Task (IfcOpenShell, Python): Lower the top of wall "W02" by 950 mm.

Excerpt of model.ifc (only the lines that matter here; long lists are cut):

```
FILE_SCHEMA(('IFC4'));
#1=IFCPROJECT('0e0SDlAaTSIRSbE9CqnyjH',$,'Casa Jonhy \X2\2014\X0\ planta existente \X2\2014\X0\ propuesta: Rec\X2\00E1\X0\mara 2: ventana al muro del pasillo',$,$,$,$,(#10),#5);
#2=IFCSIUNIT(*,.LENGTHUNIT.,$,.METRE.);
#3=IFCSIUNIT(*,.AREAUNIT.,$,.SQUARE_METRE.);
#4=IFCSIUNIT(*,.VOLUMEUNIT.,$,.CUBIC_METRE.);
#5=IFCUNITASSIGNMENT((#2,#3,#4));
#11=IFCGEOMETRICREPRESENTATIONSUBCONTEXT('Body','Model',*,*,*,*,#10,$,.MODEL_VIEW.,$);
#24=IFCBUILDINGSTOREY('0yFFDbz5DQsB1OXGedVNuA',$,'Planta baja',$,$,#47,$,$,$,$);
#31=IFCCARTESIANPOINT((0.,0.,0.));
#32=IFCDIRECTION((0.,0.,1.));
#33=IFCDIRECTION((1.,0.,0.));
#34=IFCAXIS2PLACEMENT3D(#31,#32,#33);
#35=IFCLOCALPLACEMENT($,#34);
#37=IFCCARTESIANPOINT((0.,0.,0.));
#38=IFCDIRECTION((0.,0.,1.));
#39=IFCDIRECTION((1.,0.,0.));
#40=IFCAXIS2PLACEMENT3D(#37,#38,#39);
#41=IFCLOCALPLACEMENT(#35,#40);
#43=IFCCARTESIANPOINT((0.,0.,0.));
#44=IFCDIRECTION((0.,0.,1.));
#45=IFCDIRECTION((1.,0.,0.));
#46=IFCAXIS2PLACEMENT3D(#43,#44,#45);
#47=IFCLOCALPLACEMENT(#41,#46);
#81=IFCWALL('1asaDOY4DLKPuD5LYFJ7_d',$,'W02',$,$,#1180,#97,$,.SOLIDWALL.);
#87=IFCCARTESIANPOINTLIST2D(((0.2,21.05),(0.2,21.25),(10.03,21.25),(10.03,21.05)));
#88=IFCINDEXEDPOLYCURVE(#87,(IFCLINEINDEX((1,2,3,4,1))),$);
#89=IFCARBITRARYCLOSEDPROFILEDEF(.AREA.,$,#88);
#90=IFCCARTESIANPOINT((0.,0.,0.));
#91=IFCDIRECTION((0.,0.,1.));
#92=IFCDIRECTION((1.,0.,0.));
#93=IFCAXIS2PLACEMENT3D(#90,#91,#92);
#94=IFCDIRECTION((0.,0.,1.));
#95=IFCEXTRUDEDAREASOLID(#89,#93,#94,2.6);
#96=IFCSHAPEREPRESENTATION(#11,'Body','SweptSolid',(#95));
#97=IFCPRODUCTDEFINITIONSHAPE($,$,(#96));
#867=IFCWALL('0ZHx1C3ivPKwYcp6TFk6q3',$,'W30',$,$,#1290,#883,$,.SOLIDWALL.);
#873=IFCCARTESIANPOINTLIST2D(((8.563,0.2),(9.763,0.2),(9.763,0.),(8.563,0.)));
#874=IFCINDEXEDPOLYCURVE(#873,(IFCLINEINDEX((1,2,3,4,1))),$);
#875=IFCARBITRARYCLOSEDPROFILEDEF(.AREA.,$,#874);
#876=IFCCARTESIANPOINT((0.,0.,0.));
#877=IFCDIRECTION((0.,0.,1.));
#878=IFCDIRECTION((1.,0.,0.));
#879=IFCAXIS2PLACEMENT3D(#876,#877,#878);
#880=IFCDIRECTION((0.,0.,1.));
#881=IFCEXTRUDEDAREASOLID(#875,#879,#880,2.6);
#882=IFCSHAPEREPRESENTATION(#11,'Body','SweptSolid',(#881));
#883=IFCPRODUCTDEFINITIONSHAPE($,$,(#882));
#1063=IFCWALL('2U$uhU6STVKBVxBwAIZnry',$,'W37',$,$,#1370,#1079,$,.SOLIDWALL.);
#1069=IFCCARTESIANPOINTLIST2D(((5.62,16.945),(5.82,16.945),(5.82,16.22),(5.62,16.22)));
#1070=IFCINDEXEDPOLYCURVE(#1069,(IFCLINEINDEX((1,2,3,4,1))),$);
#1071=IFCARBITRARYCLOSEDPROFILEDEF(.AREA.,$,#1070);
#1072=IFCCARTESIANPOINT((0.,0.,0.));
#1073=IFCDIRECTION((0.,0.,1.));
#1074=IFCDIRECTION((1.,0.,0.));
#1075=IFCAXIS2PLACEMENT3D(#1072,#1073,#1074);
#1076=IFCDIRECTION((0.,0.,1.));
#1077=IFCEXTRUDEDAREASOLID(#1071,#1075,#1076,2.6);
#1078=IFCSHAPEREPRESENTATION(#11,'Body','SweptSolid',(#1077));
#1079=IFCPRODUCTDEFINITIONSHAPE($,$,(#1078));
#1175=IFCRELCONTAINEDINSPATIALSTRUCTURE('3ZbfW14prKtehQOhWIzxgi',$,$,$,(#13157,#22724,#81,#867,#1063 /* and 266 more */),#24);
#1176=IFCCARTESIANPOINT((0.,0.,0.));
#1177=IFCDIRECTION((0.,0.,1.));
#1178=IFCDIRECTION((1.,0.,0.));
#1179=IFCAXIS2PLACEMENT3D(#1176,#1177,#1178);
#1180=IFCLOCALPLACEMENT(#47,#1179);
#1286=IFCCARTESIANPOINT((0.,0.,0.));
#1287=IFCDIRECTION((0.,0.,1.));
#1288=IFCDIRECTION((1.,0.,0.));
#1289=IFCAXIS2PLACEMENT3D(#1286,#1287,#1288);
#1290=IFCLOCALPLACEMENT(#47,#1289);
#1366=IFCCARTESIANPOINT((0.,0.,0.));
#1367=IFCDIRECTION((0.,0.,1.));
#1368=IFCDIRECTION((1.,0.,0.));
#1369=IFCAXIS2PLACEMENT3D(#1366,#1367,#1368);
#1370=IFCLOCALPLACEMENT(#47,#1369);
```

```python
import ifcopenshell
import ifcopenshell.geom
import ifcopenshell.util.representation
import ifcopenshell.util.shape
import ifcopenshell.util.unit

model = ifcopenshell.open("model.ifc")
unit_scale = ifcopenshell.util.unit.calculate_unit_scale(model)
settings = ifcopenshell.geom.settings()


def volume(element):
    """Net volume in cubic metres, openings subtracted."""
    shape = ifcopenshell.geom.create_shape(settings, element)
    return ifcopenshell.util.shape.get_volume(shape.geometry)


wall = model.by_guid("1asaDOY4DLKPuD5LYFJ7_d")
before = volume(wall)

body = ifcopenshell.util.representation.get_representation(wall, "Model", "Body")
solid = body.Items[0]
old_height = solid.Depth
solid.Depth -= 0.95 / unit_scale
after = volume(wall)

print(f"height {old_height:g} -> {solid.Depth:g}, volume {before:.3f} -> {after:.3f} m3")

model.write("model_rev.ifc")
```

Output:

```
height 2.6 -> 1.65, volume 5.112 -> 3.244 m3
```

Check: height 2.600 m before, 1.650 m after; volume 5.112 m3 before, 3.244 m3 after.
